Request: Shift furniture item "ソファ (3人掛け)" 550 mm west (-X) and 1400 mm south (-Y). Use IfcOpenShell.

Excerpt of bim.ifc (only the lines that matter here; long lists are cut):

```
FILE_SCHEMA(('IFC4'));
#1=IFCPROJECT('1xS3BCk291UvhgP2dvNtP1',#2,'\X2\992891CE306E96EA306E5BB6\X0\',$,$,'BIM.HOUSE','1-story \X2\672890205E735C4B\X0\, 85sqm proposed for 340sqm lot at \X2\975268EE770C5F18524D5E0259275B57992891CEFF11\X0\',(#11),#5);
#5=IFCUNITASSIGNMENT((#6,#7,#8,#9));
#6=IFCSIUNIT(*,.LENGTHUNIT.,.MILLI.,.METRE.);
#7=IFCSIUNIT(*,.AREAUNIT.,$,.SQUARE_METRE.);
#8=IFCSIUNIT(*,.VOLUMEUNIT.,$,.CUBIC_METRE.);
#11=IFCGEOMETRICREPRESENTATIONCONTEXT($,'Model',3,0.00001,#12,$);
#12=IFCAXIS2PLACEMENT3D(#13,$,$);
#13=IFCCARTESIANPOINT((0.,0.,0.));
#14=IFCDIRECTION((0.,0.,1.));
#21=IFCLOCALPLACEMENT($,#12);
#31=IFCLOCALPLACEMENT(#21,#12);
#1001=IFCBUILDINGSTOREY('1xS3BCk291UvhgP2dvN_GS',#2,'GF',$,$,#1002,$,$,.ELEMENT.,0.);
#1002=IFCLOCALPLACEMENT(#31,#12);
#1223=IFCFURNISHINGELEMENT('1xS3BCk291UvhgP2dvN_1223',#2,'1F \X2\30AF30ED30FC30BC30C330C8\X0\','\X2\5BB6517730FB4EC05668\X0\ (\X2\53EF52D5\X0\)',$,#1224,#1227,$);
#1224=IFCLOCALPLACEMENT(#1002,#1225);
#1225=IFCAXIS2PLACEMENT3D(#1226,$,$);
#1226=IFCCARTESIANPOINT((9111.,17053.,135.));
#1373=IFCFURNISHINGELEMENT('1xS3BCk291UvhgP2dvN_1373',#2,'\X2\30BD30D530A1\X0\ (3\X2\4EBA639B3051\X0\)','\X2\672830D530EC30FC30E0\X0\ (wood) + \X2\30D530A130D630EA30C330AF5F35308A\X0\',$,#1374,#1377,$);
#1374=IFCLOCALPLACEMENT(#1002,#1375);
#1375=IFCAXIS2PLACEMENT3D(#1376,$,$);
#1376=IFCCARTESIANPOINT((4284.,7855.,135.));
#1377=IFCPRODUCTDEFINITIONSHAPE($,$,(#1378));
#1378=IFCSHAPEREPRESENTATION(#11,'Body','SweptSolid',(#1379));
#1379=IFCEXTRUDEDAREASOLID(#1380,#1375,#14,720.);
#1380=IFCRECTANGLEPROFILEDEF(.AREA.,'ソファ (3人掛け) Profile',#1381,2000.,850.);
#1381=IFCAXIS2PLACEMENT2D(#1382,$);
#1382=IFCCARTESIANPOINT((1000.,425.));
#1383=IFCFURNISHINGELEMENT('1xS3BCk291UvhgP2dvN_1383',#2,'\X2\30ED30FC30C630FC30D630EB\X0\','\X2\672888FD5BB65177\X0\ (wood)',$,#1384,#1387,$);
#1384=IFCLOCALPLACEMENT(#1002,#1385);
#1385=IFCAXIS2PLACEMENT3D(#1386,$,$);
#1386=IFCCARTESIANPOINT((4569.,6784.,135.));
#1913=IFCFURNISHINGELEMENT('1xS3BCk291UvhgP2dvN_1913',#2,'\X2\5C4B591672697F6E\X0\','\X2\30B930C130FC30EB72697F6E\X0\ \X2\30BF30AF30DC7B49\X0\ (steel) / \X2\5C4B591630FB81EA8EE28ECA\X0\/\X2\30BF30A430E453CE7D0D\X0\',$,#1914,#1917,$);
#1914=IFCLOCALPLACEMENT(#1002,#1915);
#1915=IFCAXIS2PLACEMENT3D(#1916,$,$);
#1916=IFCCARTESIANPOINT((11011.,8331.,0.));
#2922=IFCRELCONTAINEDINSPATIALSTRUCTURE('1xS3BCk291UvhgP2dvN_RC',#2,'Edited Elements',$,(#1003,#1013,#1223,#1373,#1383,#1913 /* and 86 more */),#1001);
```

```python
import ifcopenshell
import ifcopenshell.api.geometry
import ifcopenshell.util.placement

model = ifcopenshell.open("bim.ifc")

item = model.by_guid("1xS3BCk291UvhgP2dvN_1373")
matrix = ifcopenshell.util.placement.get_local_placement(item.ObjectPlacement)
matrix[0, 3] -= 550.0
matrix[1, 3] -= 1400.0
ifcopenshell.api.geometry.edit_object_placement(model, product=item, matrix=matrix, is_si=False)

print(ifcopenshell.util.placement.get_local_placement(item.ObjectPlacement).round(3) + 0.0)

model.write("bim_updated.ifc")
```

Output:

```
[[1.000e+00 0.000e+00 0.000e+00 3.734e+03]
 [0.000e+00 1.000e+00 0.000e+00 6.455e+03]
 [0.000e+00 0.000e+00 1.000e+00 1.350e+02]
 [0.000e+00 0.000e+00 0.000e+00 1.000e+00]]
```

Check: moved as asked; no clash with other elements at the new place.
